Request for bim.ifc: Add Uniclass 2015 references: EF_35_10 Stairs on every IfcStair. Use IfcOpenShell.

First a look at what the model holds.

```python
import ifcopenshell

model = ifcopenshell.open("bim.ifc")
print(model.schema)
print("classifications:", [c.Name for c in model.by_type("IfcClassification")])
for ifc_class in ("IfcDoor", "IfcRoof", "IfcStair", "IfcWall", "IfcWindow"):
    print(ifc_class, len(model.by_type(ifc_class)))
```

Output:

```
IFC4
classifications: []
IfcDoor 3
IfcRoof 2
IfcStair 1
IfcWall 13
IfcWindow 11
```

```python
import ifcopenshell
import ifcopenshell.api.classification

model = ifcopenshell.open("bim.ifc")

system = ifcopenshell.api.classification.add_classification(model, classification="Uniclass 2015")

codes = {
    "IfcStair": ("EF_35_10", "Stairs"),
}
for ifc_class, (code, name) in codes.items():
    products = model.by_type(ifc_class)
    ifcopenshell.api.classification.add_reference(
        model, products=products, classification=system, identification=code, name=name
    )
    print(code, len(products))

model.write("bim_edited.ifc")
```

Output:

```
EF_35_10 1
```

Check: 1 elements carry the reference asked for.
